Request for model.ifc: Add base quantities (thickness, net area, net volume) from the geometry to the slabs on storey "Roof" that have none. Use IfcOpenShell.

First a look at what the model holds.

```python
import ifcopenshell
import ifcopenshell.util.element
import ifcopenshell.util.unit

model = ifcopenshell.open("model.ifc")
print(model.schema)
for unit_type in ("LENGTHUNIT", "AREAUNIT", "VOLUMEUNIT"):
    print(unit_type, ifcopenshell.util.unit.calculate_unit_scale(model, unit_type))
storey = next(s for s in model.by_type("IfcBuildingStorey") if s.Name == "Roof")
slabs = [e for e in ifcopenshell.util.element.get_decomposition(storey) if e.is_a("IfcSlab")]
for e in sorted(slabs, key=lambda e: e.id()):
    print(e.id(), e.is_a(), e.Name, list(ifcopenshell.util.element.get_psets(e, qtos_only=True)), sep=" | ")
```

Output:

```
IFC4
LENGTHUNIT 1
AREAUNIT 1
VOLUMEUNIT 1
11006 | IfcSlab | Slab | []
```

```python
import ifcopenshell
import ifcopenshell.api.pset
import ifcopenshell.geom
import ifcopenshell.util.element
import ifcopenshell.util.shape
import ifcopenshell.util.unit

model = ifcopenshell.open("model.ifc")
unit_scale = ifcopenshell.util.unit.calculate_unit_scale(model)
area_scale = ifcopenshell.util.unit.calculate_unit_scale(model, "AREAUNIT")
volume_scale = ifcopenshell.util.unit.calculate_unit_scale(model, "VOLUMEUNIT")
settings = ifcopenshell.geom.settings()

storey = next(s for s in model.by_type("IfcBuildingStorey") if s.Name == "Roof")
slabs = [e for e in ifcopenshell.util.element.get_decomposition(storey) if e.is_a("IfcSlab")]

for e in sorted(slabs, key=lambda e: e.id()):
    if ifcopenshell.util.element.get_psets(e, qtos_only=True, should_inherit=False):
        continue
    # Geometry comes back in metres, in the element's own axes.
    shape = ifcopenshell.geom.create_shape(settings, e)
    values = {
        "Width": ifcopenshell.util.shape.get_z(shape.geometry) / unit_scale,
        "NetArea": ifcopenshell.util.shape.get_footprint_area(shape.geometry) / area_scale,
        "NetVolume": ifcopenshell.util.shape.get_volume(shape.geometry) / volume_scale,
    }
    qto = ifcopenshell.api.pset.add_qto(model, product=e, name="Qto_SlabBaseQuantities")
    ifcopenshell.api.pset.edit_qto(model, qto=qto, properties=values)
    print(e.id(), {k: round(v, 3) for k, v in values.items()})

model.write("model_rev.ifc")
```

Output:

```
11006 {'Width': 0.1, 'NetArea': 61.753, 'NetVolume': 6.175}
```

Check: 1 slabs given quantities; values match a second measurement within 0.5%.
